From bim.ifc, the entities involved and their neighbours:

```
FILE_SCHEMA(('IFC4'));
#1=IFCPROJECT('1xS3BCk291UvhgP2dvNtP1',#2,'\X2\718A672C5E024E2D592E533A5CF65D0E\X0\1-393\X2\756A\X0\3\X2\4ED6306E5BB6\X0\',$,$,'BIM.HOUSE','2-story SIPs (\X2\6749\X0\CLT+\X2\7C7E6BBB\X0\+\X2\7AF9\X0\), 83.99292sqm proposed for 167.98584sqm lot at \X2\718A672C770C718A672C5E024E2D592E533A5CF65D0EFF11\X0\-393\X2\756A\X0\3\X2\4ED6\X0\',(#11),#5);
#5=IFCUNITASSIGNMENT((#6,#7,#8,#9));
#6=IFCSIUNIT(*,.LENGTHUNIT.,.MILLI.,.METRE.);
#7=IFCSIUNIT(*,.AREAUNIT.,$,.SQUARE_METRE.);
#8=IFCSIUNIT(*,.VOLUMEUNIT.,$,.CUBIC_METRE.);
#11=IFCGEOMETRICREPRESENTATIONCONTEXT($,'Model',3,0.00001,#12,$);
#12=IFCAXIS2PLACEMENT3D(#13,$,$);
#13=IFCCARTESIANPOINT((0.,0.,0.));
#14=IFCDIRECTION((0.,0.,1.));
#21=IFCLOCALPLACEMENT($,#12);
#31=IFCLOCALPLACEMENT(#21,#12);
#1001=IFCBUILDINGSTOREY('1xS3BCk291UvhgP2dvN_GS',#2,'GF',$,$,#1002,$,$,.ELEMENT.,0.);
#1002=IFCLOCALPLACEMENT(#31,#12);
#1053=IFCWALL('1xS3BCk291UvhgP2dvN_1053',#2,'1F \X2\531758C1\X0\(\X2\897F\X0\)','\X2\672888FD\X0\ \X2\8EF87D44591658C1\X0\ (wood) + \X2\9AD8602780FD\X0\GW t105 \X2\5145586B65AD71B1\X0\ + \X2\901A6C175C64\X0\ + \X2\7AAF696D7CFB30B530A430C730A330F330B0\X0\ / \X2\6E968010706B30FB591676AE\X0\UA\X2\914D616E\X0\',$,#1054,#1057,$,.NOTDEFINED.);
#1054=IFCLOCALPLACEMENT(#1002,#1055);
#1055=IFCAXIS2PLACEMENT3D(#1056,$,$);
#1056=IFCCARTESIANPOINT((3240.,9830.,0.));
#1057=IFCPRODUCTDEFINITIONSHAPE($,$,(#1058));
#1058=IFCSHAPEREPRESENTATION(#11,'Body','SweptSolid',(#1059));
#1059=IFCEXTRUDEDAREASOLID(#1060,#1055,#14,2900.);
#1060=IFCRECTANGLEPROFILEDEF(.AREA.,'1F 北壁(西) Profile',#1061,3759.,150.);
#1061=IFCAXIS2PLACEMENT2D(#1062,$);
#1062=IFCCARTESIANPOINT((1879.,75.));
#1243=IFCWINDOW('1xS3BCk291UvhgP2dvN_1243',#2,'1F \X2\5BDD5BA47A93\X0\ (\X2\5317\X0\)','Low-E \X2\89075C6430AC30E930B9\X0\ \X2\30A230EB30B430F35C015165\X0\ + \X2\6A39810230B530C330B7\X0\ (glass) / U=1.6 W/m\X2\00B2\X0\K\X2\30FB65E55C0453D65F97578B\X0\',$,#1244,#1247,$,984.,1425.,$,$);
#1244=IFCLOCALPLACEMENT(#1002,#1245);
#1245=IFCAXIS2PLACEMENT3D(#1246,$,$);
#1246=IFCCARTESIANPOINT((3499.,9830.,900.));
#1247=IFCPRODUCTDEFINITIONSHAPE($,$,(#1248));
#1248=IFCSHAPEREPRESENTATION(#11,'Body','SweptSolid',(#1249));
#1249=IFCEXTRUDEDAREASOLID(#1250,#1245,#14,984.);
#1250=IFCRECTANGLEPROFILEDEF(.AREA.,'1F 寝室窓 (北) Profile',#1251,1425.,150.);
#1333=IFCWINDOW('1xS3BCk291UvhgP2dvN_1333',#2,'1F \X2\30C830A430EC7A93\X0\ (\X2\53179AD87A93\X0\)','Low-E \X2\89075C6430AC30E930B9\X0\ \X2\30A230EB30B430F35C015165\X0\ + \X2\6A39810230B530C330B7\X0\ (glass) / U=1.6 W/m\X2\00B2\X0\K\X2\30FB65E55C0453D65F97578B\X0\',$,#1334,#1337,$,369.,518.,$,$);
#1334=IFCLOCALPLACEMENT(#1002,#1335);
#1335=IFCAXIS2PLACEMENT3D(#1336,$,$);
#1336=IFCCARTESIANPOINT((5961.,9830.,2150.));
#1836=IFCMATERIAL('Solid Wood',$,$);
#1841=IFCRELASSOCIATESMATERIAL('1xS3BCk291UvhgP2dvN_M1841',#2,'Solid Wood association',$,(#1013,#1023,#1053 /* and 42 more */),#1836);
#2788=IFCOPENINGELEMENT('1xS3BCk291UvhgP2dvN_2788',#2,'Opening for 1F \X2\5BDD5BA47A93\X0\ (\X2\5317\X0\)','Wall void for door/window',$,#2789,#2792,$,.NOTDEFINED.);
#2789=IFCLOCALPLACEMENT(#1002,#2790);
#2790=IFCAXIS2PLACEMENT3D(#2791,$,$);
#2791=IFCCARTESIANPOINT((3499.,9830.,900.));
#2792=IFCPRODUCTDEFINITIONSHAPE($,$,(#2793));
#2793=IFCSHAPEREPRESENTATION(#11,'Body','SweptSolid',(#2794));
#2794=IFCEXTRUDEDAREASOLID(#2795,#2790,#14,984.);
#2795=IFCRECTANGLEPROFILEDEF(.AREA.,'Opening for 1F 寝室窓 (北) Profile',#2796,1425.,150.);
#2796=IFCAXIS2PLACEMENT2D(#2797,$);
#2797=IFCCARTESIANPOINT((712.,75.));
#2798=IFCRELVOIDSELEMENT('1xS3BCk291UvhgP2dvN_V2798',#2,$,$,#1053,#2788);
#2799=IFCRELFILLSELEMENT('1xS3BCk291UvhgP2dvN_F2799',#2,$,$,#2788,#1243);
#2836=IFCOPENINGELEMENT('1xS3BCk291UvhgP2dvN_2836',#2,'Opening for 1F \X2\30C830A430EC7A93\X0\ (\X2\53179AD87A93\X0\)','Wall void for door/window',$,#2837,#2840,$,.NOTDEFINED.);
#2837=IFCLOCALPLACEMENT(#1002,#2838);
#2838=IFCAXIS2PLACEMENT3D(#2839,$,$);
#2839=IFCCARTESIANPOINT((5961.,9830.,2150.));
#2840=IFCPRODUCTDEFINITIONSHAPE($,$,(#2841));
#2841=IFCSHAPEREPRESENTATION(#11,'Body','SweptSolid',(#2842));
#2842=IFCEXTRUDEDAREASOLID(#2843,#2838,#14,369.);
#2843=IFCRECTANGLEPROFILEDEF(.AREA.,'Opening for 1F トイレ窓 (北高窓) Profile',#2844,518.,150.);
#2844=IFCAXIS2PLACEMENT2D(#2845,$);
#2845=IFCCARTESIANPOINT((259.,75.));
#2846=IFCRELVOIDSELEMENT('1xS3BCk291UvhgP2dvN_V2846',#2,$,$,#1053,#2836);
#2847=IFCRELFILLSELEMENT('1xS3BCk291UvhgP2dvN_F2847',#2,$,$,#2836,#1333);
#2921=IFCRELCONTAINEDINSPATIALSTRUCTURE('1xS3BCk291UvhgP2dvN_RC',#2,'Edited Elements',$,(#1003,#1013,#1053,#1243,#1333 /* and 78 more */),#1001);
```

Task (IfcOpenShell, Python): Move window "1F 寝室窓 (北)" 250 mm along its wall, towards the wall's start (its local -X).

```python
import ifcopenshell
import ifcopenshell.api.geometry
import ifcopenshell.util.placement

model = ifcopenshell.open("bim.ifc")

window = model.by_guid("1xS3BCk291UvhgP2dvN_1243")
opening = window.FillsVoids[0].RelatingOpeningElement
wall = opening.VoidsElements[0].RelatingBuildingElement

wall_matrix = ifcopenshell.util.placement.get_local_placement(wall.ObjectPlacement)
shift = wall_matrix[:3, 0] * -250.0
before = ifcopenshell.util.placement.get_local_placement(window.ObjectPlacement)[:3, 3].copy()

# The window is not placed relative to its opening, so move both.
for product in (opening, window):
    matrix = ifcopenshell.util.placement.get_local_placement(product.ObjectPlacement)
    matrix[:3, 3] += shift
    ifcopenshell.api.geometry.edit_object_placement(model, product=product, matrix=matrix, is_si=False)

after = ifcopenshell.util.placement.get_local_placement(window.ObjectPlacement)[:3, 3]
print("window moved by", (after - before).round(3) + 0.0)

model.write("bim-out.ifc")
```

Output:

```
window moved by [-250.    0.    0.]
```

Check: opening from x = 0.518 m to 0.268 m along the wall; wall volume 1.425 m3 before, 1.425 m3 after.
